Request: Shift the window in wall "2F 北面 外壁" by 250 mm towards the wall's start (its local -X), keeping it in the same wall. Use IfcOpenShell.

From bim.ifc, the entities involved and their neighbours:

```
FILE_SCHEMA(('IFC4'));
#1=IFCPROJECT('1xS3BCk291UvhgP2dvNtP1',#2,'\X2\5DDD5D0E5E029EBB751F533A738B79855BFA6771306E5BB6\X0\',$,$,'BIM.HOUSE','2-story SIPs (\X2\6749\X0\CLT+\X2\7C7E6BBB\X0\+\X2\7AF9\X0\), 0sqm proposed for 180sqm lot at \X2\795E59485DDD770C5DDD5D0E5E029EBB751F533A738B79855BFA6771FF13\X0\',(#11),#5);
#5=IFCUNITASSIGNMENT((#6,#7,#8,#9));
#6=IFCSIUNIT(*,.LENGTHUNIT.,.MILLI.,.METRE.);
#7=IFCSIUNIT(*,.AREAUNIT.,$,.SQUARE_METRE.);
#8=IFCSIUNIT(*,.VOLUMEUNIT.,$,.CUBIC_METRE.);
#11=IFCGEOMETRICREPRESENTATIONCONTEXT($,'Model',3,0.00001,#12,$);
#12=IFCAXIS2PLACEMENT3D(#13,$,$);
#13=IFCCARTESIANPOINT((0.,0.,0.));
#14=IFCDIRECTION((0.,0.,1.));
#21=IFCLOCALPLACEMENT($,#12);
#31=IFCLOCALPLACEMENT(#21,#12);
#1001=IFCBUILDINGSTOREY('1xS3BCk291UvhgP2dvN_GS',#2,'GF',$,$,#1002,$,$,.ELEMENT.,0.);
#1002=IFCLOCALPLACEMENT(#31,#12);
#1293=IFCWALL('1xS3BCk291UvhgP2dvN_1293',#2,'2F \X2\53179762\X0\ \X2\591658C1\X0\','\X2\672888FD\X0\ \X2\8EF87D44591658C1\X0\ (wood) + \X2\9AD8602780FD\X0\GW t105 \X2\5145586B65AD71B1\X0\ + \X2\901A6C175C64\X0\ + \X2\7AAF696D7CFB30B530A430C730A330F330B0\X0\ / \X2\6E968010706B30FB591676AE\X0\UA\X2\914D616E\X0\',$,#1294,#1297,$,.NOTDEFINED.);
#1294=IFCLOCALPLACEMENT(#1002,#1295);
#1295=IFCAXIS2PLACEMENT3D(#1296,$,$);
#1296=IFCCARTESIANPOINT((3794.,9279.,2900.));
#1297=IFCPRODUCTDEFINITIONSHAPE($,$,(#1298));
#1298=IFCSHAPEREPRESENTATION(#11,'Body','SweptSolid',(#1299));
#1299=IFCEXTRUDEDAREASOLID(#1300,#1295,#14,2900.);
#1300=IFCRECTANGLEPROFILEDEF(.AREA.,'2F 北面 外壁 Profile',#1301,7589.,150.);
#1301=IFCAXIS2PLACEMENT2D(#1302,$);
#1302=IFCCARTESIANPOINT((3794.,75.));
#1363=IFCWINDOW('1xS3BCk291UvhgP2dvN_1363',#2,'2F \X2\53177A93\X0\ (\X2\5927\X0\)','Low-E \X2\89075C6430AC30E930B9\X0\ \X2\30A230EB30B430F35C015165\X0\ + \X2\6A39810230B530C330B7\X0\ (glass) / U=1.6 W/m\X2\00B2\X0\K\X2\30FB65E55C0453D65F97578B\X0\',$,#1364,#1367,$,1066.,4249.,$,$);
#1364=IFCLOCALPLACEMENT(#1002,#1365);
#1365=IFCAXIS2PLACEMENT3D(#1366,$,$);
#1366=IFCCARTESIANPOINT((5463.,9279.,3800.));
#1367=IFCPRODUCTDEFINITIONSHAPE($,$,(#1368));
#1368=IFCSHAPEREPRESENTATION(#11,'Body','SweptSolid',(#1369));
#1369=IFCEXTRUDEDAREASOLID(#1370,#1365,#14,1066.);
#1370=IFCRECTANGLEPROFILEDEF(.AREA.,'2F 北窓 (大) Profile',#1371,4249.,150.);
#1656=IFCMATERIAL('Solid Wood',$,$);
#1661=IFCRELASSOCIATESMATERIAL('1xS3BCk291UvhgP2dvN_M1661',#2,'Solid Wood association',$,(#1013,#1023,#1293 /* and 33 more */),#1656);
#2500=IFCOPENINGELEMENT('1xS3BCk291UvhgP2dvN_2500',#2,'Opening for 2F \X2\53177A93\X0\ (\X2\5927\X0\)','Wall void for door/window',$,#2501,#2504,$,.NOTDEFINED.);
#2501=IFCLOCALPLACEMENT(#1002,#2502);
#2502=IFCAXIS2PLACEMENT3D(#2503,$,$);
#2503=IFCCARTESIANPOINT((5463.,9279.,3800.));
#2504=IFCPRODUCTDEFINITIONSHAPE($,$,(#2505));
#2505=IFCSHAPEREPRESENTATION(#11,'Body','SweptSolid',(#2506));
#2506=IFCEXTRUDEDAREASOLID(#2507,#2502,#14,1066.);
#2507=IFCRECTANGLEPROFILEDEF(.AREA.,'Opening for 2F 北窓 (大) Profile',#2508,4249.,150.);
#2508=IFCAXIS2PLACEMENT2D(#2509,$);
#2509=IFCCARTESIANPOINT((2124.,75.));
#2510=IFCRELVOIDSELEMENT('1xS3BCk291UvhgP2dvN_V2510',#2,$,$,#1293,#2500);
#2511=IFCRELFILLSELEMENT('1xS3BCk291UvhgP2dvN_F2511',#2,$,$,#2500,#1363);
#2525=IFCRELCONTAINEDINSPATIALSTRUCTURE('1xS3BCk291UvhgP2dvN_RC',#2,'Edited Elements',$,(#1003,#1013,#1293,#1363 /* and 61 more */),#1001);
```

```python
import ifcopenshell
import ifcopenshell.api.geometry
import ifcopenshell.util.placement

model = ifcopenshell.open("bim.ifc")

window = model.by_guid("1xS3BCk291UvhgP2dvN_1363")
opening = window.FillsVoids[0].RelatingOpeningElement
wall = opening.VoidsElements[0].RelatingBuildingElement

wall_matrix = ifcopenshell.util.placement.get_local_placement(wall.ObjectPlacement)
shift = wall_matrix[:3, 0] * -250.0
before = ifcopenshell.util.placement.get_local_placement(window.ObjectPlacement)[:3, 3].copy()

# The window is not placed relative to its opening, so move both.
for product in (opening, window):
    matrix = ifcopenshell.util.placement.get_local_placement(product.ObjectPlacement)
    matrix[:3, 3] += shift
    ifcopenshell.api.geometry.edit_object_placement(model, product=product, matrix=matrix, is_si=False)

after = ifcopenshell.util.placement.get_local_placement(window.ObjectPlacement)[:3, 3]
print("window moved by", (after - before).round(3) + 0.0)

model.write("bim_rev.ifc")
```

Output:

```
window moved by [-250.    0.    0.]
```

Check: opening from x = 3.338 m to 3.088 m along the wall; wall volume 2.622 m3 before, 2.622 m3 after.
